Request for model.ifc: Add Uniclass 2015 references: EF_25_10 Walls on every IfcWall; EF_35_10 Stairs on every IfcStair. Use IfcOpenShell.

First a look at what the model holds.

```python
import ifcopenshell

model = ifcopenshell.open("model.ifc")
print(model.schema)
print("classifications:", [c.Name for c in model.by_type("IfcClassification")])
for ifc_class in ("IfcDoor", "IfcRoof", "IfcStair", "IfcWall", "IfcWindow"):
    print(ifc_class, len(model.by_type(ifc_class)))
```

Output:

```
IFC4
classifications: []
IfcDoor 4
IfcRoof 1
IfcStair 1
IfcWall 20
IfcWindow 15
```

```python
import ifcopenshell
import ifcopenshell.api.classification

model = ifcopenshell.open("model.ifc")

system = ifcopenshell.api.classification.add_classification(model, classification="Uniclass 2015")

codes = {
    "IfcWall": ("EF_25_10", "Walls"),
    "IfcStair": ("EF_35_10", "Stairs"),
}
for ifc_class, (code, name) in codes.items():
    products = model.by_type(ifc_class)
    ifcopenshell.api.classification.add_reference(
        model, products=products, classification=system, identification=code, name=name
    )
    print(code, len(products))

model.write("model_edited.ifc")
```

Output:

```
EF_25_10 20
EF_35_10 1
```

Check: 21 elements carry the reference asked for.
